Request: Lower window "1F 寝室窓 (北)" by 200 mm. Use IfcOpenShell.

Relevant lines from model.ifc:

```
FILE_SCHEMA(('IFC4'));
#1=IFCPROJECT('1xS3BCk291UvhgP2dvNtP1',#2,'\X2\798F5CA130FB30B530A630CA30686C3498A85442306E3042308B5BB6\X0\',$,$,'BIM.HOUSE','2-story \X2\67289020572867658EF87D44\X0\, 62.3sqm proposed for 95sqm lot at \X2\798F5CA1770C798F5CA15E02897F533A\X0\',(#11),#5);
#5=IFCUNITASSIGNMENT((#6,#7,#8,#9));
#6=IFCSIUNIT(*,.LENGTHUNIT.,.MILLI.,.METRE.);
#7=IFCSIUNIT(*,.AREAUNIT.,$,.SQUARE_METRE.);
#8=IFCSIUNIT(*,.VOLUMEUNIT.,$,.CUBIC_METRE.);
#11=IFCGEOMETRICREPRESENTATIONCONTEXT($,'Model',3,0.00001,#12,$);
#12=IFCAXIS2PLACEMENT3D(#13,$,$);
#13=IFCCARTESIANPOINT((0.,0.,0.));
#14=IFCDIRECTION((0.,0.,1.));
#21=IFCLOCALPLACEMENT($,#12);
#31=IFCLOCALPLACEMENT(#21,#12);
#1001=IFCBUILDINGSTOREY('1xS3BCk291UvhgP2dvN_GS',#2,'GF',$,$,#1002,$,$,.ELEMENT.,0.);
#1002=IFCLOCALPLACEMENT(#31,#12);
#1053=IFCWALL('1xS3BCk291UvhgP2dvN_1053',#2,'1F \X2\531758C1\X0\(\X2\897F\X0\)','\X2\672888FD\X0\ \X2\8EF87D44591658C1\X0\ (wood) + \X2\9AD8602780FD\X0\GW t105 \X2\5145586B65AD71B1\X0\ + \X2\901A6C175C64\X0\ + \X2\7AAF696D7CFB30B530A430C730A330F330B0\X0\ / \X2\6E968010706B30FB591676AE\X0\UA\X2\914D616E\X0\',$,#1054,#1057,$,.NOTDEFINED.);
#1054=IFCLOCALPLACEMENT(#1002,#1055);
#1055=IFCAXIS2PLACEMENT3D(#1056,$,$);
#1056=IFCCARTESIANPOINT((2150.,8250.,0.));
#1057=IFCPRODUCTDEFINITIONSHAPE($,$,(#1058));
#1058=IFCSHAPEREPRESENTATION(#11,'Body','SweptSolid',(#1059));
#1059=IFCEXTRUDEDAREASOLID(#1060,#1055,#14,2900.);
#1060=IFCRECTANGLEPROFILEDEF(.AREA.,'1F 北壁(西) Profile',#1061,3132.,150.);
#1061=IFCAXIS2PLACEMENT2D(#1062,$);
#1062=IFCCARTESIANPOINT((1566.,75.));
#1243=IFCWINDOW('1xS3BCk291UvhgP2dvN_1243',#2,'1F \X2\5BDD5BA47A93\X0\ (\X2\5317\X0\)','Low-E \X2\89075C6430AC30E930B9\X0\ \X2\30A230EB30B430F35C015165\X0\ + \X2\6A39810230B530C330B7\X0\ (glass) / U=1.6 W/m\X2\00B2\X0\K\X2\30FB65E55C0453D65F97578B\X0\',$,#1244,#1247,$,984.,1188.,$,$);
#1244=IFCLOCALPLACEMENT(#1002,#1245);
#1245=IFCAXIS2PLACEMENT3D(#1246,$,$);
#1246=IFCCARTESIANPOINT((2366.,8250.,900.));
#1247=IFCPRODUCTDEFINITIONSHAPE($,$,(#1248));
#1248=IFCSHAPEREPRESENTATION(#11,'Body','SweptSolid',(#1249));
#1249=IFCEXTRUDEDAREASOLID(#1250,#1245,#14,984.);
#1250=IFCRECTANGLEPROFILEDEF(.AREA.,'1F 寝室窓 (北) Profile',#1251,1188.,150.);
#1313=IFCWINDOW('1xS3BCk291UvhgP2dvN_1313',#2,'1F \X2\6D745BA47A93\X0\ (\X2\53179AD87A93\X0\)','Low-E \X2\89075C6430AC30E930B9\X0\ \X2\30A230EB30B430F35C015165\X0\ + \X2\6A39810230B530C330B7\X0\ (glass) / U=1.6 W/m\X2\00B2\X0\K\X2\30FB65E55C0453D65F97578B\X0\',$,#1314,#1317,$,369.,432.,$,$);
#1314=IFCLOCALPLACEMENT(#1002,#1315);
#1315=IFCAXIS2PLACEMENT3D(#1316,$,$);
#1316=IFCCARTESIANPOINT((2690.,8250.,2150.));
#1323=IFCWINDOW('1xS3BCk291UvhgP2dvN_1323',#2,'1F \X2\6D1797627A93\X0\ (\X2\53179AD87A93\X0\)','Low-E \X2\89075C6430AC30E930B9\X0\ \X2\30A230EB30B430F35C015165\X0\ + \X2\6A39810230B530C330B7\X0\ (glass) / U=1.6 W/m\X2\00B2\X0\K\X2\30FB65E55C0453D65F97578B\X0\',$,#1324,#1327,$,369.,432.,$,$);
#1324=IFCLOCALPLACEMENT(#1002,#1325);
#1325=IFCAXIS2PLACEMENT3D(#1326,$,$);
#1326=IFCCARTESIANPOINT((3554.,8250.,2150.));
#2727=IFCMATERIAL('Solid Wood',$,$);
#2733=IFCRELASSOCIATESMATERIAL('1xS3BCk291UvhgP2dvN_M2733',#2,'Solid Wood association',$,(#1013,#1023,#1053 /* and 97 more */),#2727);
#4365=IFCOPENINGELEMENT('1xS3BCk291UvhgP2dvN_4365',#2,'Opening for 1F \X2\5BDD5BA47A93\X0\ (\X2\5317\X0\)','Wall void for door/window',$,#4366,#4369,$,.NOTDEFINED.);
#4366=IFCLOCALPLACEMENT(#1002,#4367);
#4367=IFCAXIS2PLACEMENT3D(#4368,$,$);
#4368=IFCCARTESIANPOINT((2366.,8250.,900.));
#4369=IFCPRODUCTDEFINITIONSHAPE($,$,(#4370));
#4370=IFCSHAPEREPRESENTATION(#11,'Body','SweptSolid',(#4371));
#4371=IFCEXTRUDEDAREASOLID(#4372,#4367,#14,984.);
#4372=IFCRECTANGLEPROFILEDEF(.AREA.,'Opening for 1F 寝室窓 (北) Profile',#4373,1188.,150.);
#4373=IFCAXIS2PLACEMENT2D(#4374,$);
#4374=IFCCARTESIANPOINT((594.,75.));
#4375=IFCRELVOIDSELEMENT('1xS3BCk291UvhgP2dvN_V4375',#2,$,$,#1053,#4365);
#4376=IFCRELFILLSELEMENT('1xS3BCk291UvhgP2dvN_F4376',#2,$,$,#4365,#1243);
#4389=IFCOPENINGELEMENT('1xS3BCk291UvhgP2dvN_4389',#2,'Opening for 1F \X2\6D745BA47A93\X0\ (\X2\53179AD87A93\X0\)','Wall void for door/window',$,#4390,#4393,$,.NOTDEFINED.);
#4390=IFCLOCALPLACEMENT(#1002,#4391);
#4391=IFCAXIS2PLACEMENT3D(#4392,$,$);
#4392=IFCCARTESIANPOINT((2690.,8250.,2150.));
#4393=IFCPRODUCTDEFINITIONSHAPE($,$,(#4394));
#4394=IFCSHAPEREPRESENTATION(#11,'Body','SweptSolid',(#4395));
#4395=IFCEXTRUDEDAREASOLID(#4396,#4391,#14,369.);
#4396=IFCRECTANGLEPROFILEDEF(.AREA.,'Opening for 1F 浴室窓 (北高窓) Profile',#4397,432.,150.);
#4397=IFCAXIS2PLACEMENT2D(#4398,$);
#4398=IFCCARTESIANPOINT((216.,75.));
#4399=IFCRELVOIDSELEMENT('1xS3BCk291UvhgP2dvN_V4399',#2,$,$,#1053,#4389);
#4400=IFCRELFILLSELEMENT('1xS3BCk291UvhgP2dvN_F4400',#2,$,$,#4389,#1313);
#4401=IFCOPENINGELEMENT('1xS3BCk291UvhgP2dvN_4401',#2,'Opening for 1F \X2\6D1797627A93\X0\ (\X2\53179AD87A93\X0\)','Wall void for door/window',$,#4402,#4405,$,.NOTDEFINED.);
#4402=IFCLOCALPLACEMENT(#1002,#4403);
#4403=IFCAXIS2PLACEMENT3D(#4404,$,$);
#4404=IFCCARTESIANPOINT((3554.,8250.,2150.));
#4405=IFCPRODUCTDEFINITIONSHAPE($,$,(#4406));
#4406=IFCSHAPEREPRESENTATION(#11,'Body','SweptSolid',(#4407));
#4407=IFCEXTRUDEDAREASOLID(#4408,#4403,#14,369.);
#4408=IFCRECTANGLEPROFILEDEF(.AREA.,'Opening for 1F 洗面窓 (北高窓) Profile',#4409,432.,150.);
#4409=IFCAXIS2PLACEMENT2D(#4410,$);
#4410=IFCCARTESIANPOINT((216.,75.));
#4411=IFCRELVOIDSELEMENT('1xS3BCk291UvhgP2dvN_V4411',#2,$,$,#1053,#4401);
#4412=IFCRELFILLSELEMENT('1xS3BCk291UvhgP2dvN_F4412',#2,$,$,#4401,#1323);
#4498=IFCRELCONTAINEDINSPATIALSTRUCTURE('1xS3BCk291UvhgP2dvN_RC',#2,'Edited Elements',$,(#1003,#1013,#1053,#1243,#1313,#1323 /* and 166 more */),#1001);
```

```python
import numpy as np
import ifcopenshell
import ifcopenshell.api.geometry
import ifcopenshell.util.placement
import ifcopenshell.util.unit

model = ifcopenshell.open("model.ifc")
unit_scale = ifcopenshell.util.unit.calculate_unit_scale(model)

window = model.by_guid("1xS3BCk291UvhgP2dvN_1243")
opening = window.FillsVoids[0].RelatingOpeningElement
dz = -0.2 / unit_scale

shift = np.array([0.0, 0.0, dz])
# The window is not placed relative to its opening, so move both.
for product in (opening, window):
    matrix = ifcopenshell.util.placement.get_local_placement(product.ObjectPlacement)
    matrix[:3, 3] += shift
    ifcopenshell.api.geometry.edit_object_placement(model, product=product, matrix=matrix, is_si=False)

print(f"moved by {dz * unit_scale:+.3f} m")

model.write("model-out.ifc")
```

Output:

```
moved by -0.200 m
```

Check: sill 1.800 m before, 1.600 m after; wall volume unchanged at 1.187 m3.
